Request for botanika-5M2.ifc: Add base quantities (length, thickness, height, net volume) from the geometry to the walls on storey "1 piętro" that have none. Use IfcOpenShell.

First a look at what the model holds.

```python
import ifcopenshell
import ifcopenshell.util.element
import ifcopenshell.util.unit

model = ifcopenshell.open("botanika-5M2.ifc")
print(model.schema)
for unit_type in ("LENGTHUNIT", "AREAUNIT", "VOLUMEUNIT"):
    print(unit_type, ifcopenshell.util.unit.calculate_unit_scale(model, unit_type))
storey = next(s for s in model.by_type("IfcBuildingStorey") if s.Name == "1 piętro")
walls = [e for e in ifcopenshell.util.element.get_decomposition(storey) if e.is_a("IfcWall")]
for e in sorted(walls, key=lambda e: e.id()):
    print(e.id(), e.is_a(), e.Name, list(ifcopenshell.util.element.get_psets(e, qtos_only=True)), sep=" | ")
```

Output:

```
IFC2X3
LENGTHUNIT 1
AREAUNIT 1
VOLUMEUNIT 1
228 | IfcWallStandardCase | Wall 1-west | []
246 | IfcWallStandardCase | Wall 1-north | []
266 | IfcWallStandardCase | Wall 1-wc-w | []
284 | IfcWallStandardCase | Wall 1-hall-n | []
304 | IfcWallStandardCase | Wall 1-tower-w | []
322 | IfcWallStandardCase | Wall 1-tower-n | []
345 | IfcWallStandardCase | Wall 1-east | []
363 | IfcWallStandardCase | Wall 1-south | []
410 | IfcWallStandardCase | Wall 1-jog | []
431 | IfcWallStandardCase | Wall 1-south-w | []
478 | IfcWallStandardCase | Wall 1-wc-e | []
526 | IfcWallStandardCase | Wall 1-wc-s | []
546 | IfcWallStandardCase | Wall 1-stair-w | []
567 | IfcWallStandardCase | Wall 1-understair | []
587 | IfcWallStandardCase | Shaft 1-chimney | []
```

```python
import ifcopenshell
import ifcopenshell.api.pset
import ifcopenshell.geom
import ifcopenshell.util.element
import ifcopenshell.util.shape
import ifcopenshell.util.unit

model = ifcopenshell.open("botanika-5M2.ifc")
unit_scale = ifcopenshell.util.unit.calculate_unit_scale(model)
volume_scale = ifcopenshell.util.unit.calculate_unit_scale(model, "VOLUMEUNIT")
settings = ifcopenshell.geom.settings()

storey = next(s for s in model.by_type("IfcBuildingStorey") if s.Name == "1 piętro")
walls = [e for e in ifcopenshell.util.element.get_decomposition(storey) if e.is_a("IfcWall")]

for e in sorted(walls, key=lambda e: e.id()):
    if ifcopenshell.util.element.get_psets(e, qtos_only=True, should_inherit=False):
        continue
    # Geometry comes back in metres, in the element's own axes.
    shape = ifcopenshell.geom.create_shape(settings, e)
    values = {
        "Length": ifcopenshell.util.shape.get_x(shape.geometry) / unit_scale,
        "Width": ifcopenshell.util.shape.get_y(shape.geometry) / unit_scale,
        "Height": ifcopenshell.util.shape.get_z(shape.geometry) / unit_scale,
        "NetVolume": ifcopenshell.util.shape.get_volume(shape.geometry) / volume_scale,
    }
    qto = ifcopenshell.api.pset.add_qto(model, product=e, name="BaseQuantities")
    ifcopenshell.api.pset.edit_qto(model, qto=qto, properties=values)
    print(e.id(), {k: round(v, 3) for k, v in values.items()})

model.write("botanika-5M2_v2.ifc")
```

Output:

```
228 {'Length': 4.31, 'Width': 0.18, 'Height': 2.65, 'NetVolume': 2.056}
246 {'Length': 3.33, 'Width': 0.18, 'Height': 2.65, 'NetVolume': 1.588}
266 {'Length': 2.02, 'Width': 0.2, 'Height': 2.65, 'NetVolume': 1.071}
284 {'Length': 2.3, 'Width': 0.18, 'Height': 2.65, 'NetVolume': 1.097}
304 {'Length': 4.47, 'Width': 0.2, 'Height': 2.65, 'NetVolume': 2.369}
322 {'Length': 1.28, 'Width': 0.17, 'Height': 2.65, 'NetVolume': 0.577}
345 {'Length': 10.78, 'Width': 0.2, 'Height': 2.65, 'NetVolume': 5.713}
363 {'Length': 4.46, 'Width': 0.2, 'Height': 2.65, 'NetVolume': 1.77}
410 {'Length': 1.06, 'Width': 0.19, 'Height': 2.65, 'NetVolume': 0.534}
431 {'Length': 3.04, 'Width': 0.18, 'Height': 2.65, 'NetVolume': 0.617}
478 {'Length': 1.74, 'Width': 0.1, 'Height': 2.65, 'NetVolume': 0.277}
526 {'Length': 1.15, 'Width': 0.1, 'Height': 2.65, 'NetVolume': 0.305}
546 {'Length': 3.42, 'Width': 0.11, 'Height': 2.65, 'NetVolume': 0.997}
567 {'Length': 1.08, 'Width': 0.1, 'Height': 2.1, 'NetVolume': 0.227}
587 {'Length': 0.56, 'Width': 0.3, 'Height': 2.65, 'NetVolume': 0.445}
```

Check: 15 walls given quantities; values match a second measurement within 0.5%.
